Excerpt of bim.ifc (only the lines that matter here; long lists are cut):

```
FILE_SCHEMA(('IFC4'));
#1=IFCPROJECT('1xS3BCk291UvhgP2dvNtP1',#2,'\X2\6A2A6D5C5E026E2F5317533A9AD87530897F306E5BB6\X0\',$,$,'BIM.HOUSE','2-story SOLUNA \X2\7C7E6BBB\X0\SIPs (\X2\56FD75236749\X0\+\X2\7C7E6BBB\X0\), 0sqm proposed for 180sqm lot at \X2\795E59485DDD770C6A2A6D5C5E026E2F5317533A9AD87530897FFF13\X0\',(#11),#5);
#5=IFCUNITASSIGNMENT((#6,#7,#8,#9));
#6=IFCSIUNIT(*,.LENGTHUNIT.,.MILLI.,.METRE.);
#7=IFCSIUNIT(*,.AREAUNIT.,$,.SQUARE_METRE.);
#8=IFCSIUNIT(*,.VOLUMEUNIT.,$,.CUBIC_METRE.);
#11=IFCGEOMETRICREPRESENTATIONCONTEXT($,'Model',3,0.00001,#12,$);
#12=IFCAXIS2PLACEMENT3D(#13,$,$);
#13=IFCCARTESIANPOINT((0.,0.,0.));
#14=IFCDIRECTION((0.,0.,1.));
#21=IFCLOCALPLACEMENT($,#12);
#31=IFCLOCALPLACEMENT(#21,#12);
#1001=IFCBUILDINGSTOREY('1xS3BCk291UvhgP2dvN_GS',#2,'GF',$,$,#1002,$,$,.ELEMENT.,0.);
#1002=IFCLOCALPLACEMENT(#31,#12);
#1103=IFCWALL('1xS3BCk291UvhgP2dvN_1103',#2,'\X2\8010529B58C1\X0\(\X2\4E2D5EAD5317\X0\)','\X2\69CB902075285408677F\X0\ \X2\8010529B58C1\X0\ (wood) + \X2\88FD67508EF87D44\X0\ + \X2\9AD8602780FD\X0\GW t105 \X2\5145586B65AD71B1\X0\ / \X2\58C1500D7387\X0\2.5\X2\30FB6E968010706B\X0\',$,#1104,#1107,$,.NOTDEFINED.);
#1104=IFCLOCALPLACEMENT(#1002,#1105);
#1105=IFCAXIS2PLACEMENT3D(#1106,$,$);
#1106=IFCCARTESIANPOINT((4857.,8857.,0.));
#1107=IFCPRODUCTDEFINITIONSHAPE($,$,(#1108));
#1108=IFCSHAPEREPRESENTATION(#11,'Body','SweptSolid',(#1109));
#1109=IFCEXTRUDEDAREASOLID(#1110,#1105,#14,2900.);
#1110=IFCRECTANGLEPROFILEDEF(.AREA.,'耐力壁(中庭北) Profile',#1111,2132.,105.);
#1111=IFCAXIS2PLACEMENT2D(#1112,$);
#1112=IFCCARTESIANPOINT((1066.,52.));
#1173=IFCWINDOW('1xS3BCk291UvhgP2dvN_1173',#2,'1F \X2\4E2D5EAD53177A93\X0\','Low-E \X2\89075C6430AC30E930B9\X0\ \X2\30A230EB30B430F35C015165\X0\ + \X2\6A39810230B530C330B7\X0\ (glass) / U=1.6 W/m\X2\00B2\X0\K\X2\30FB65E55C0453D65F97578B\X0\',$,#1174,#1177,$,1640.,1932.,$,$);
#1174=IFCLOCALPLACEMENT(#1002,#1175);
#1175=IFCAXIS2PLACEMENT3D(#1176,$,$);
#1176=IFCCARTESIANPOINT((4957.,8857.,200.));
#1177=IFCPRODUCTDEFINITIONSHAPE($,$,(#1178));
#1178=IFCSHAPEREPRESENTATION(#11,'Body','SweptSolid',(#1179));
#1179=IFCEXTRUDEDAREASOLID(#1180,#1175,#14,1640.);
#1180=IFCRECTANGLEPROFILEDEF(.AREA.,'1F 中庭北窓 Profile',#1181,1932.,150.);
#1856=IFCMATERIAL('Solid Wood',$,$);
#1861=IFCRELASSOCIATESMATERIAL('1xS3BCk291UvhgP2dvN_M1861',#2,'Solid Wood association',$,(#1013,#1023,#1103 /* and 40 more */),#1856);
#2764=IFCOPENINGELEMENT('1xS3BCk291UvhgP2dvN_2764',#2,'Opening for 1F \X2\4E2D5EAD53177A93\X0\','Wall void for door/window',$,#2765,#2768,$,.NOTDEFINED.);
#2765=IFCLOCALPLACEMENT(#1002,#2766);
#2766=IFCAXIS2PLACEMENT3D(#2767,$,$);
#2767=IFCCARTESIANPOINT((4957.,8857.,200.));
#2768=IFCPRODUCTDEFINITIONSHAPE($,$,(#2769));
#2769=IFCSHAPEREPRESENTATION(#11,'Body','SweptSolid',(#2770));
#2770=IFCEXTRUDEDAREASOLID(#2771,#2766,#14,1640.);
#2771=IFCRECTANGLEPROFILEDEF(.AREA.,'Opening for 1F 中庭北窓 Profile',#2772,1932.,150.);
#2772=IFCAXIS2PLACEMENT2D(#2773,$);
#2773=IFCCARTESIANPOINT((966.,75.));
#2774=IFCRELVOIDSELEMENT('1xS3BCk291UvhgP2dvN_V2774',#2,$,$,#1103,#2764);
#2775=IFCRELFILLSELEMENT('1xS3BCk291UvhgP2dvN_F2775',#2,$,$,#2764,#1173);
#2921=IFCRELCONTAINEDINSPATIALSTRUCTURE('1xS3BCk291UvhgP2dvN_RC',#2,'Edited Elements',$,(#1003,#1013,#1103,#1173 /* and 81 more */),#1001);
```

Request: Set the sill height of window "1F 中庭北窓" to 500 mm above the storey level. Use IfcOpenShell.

```python
import numpy as np
import ifcopenshell
import ifcopenshell.api.geometry
import ifcopenshell.geom
import ifcopenshell.util.element
import ifcopenshell.util.placement
import ifcopenshell.util.shape
import ifcopenshell.util.unit

model = ifcopenshell.open("bim.ifc")
unit_scale = ifcopenshell.util.unit.calculate_unit_scale(model)

window = model.by_guid("1xS3BCk291UvhgP2dvN_1173")
opening = window.FillsVoids[0].RelatingOpeningElement
storey = ifcopenshell.util.element.get_container(window, ifc_class="IfcBuildingStorey")
level = ifcopenshell.util.placement.get_local_placement(storey.ObjectPlacement)[2, 3]

# The opening's origin need not be at the sill, so measure its lowest point.
shape = ifcopenshell.geom.create_shape(ifcopenshell.geom.settings(), opening)
bottom = ifcopenshell.util.shape.get_shape_bottom_elevation(shape, shape.geometry) / unit_scale
dz = level + 500.0 - bottom

shift = np.array([0.0, 0.0, dz])
# The window is not placed relative to its opening, so move both.
for product in (opening, window):
    matrix = ifcopenshell.util.placement.get_local_placement(product.ObjectPlacement)
    matrix[:3, 3] += shift
    ifcopenshell.api.geometry.edit_object_placement(model, product=product, matrix=matrix, is_si=False)

print(f"moved by {dz * unit_scale:+.3f} m")

model.write("bim_edited.ifc")
```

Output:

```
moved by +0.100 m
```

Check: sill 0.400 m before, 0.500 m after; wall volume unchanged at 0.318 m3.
